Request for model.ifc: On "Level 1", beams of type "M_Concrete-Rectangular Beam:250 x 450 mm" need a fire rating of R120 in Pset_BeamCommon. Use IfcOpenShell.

First a look at what the model holds.

```python
import ifcopenshell
import ifcopenshell.util.element

model = ifcopenshell.open("model.ifc")
print(model.schema)
storey = next(s for s in model.by_type("IfcBuildingStorey") if s.Name == "Level 1")
beams = [e for e in ifcopenshell.util.element.get_decomposition(storey) if e.is_a("IfcBeam")]
seen = {}
for e in beams:
    element_type = ifcopenshell.util.element.get_type(e)
    key = (element_type.Name if element_type != e and element_type else None, ifcopenshell.util.element.get_pset(e, "Pset_BeamCommon", "FireRating"))
    seen[key] = seen.get(key, 0) + 1
for (name, value), count in sorted(seen.items(), key=str):
    print(count, "x", name, "|", value)
```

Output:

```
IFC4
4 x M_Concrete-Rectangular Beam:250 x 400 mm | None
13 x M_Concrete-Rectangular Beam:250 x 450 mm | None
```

```python
import ifcopenshell
import ifcopenshell.api.pset
import ifcopenshell.util.element

model = ifcopenshell.open("model.ifc")

storey = next(s for s in model.by_type("IfcBuildingStorey") if s.Name == "Level 1")
beams = [e for e in ifcopenshell.util.element.get_decomposition(storey) if e.is_a("IfcBeam")]

count = 0
for e in beams:
    element_type = ifcopenshell.util.element.get_type(e)
    if element_type in (None, e) or element_type.Name != "M_Concrete-Rectangular Beam:250 x 450 mm":
        continue
    # add_pset returns the element's existing set when there is one.
    pset = ifcopenshell.api.pset.add_pset(model, product=e, name="Pset_BeamCommon")
    ifcopenshell.api.pset.edit_pset(model, pset=pset, properties={"FireRating": "R120"})
    count += 1

print(count, "beams updated")

model.write("model_updated.ifc")
```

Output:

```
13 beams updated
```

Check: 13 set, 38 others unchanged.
